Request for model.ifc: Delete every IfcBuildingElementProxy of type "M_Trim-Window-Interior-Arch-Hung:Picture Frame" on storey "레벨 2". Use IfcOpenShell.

First a look at what the model holds.

```python
import ifcopenshell
import ifcopenshell.util.element

model = ifcopenshell.open("model.ifc")
print(model.schema)
storey = next(s for s in model.by_type("IfcBuildingStorey") if s.Name == "레벨 2")
proxies = [e for e in ifcopenshell.util.element.get_decomposition(storey) if e.is_a("IfcBuildingElementProxy")]
seen = {}
for e in proxies:
    element_type = ifcopenshell.util.element.get_type(e)
    name = element_type.Name if element_type not in (None, e) else None
    seen[name] = seen.get(name, 0) + 1
for name, count in sorted(seen.items(), key=str):
    print(count, "x", name)
```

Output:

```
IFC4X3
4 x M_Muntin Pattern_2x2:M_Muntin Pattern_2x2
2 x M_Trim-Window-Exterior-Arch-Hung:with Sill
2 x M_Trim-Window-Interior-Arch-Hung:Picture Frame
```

```python
import ifcopenshell
import ifcopenshell.api.root
import ifcopenshell.util.element

model = ifcopenshell.open("model.ifc")

storey = next(s for s in model.by_type("IfcBuildingStorey") if s.Name == "레벨 2")
proxies = [e for e in ifcopenshell.util.element.get_decomposition(storey) if e.is_a("IfcBuildingElementProxy")]
targets = [e for e in proxies if (t := ifcopenshell.util.element.get_type(e)) not in (None, e) and t.Name == "M_Trim-Window-Interior-Arch-Hung:Picture Frame"]

for e in targets:
    ifcopenshell.api.root.remove_product(model, product=e)
print(len(targets), "removed")

model.write("model_updated.ifc")
```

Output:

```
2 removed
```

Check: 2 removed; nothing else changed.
